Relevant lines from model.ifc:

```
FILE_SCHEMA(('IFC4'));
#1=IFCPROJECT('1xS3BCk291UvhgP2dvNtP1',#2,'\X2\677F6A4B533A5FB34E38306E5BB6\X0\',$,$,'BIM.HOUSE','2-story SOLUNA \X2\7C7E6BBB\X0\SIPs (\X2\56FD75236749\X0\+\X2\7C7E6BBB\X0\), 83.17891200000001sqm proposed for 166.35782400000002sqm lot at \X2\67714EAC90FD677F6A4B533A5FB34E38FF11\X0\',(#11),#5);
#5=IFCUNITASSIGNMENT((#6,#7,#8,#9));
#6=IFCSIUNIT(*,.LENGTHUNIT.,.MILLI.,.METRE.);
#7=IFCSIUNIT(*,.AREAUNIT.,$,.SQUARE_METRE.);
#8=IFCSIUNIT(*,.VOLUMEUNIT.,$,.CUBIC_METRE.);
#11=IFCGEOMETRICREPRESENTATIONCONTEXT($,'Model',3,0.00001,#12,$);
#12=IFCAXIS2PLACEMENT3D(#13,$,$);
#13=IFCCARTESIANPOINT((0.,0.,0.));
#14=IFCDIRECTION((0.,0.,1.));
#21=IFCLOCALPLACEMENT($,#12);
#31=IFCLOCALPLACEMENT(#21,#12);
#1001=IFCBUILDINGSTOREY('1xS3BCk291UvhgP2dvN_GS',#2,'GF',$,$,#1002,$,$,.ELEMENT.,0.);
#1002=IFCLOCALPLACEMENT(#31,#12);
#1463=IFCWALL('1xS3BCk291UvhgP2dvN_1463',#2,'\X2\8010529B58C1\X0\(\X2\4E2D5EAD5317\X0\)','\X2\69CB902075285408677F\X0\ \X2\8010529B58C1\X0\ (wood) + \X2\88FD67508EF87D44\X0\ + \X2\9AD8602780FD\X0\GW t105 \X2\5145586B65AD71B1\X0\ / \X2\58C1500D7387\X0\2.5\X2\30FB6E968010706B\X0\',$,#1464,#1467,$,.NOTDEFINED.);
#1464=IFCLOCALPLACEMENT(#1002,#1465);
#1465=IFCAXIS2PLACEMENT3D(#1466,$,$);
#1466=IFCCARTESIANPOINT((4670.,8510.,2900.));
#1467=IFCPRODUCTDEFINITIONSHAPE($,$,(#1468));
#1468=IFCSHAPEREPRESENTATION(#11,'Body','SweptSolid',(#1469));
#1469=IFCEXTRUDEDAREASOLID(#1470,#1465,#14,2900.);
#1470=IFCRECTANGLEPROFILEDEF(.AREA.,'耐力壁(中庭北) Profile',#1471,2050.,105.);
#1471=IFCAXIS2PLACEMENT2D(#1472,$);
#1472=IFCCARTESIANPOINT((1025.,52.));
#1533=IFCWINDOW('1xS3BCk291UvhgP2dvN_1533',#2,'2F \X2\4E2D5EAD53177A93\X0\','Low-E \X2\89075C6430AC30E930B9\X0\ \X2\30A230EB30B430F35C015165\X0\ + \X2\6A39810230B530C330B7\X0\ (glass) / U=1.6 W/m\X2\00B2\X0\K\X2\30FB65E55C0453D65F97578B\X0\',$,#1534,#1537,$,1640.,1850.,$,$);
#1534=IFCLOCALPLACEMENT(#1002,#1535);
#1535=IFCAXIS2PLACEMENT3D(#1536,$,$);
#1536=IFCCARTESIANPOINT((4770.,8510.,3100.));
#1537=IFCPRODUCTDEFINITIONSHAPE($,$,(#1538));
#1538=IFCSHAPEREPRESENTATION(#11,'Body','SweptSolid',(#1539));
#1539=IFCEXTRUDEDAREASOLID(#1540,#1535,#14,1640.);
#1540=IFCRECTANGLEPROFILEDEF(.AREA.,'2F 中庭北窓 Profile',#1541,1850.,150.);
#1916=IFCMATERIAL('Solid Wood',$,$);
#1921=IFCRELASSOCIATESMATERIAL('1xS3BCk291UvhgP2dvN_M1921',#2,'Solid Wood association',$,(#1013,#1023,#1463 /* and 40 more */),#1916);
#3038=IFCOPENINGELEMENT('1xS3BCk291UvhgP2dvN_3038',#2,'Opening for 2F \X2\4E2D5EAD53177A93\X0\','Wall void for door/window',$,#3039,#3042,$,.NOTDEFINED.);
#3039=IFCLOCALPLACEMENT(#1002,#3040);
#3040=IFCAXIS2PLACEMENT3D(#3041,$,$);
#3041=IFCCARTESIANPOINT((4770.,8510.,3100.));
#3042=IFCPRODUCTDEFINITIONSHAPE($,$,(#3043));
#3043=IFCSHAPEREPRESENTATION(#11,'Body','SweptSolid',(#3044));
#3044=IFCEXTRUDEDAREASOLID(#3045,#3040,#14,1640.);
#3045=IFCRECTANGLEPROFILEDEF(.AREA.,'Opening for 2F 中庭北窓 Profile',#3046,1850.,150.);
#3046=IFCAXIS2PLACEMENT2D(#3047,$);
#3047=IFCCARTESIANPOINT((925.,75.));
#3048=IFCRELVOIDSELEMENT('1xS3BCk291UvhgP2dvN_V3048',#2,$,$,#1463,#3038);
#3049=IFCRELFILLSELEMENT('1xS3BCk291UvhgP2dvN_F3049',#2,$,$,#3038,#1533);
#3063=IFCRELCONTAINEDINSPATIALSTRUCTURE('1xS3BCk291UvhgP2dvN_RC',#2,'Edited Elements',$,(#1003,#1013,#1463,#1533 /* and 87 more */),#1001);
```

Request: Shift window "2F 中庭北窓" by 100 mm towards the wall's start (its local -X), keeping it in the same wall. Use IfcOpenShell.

```python
import ifcopenshell
import ifcopenshell.api.geometry
import ifcopenshell.util.placement

model = ifcopenshell.open("model.ifc")

window = model.by_guid("1xS3BCk291UvhgP2dvN_1533")
opening = window.FillsVoids[0].RelatingOpeningElement
wall = opening.VoidsElements[0].RelatingBuildingElement

wall_matrix = ifcopenshell.util.placement.get_local_placement(wall.ObjectPlacement)
shift = wall_matrix[:3, 0] * -100.0
before = ifcopenshell.util.placement.get_local_placement(window.ObjectPlacement)[:3, 3].copy()

# The window is not placed relative to its opening, so move both.
for product in (opening, window):
    matrix = ifcopenshell.util.placement.get_local_placement(product.ObjectPlacement)
    matrix[:3, 3] += shift
    ifcopenshell.api.geometry.edit_object_placement(model, product=product, matrix=matrix, is_si=False)

after = ifcopenshell.util.placement.get_local_placement(window.ObjectPlacement)[:3, 3]
print("window moved by", (after - before).round(3) + 0.0)

model.write("model_rev.ifc")
```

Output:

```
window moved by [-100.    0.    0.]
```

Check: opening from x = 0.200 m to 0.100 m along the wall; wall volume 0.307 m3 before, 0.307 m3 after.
